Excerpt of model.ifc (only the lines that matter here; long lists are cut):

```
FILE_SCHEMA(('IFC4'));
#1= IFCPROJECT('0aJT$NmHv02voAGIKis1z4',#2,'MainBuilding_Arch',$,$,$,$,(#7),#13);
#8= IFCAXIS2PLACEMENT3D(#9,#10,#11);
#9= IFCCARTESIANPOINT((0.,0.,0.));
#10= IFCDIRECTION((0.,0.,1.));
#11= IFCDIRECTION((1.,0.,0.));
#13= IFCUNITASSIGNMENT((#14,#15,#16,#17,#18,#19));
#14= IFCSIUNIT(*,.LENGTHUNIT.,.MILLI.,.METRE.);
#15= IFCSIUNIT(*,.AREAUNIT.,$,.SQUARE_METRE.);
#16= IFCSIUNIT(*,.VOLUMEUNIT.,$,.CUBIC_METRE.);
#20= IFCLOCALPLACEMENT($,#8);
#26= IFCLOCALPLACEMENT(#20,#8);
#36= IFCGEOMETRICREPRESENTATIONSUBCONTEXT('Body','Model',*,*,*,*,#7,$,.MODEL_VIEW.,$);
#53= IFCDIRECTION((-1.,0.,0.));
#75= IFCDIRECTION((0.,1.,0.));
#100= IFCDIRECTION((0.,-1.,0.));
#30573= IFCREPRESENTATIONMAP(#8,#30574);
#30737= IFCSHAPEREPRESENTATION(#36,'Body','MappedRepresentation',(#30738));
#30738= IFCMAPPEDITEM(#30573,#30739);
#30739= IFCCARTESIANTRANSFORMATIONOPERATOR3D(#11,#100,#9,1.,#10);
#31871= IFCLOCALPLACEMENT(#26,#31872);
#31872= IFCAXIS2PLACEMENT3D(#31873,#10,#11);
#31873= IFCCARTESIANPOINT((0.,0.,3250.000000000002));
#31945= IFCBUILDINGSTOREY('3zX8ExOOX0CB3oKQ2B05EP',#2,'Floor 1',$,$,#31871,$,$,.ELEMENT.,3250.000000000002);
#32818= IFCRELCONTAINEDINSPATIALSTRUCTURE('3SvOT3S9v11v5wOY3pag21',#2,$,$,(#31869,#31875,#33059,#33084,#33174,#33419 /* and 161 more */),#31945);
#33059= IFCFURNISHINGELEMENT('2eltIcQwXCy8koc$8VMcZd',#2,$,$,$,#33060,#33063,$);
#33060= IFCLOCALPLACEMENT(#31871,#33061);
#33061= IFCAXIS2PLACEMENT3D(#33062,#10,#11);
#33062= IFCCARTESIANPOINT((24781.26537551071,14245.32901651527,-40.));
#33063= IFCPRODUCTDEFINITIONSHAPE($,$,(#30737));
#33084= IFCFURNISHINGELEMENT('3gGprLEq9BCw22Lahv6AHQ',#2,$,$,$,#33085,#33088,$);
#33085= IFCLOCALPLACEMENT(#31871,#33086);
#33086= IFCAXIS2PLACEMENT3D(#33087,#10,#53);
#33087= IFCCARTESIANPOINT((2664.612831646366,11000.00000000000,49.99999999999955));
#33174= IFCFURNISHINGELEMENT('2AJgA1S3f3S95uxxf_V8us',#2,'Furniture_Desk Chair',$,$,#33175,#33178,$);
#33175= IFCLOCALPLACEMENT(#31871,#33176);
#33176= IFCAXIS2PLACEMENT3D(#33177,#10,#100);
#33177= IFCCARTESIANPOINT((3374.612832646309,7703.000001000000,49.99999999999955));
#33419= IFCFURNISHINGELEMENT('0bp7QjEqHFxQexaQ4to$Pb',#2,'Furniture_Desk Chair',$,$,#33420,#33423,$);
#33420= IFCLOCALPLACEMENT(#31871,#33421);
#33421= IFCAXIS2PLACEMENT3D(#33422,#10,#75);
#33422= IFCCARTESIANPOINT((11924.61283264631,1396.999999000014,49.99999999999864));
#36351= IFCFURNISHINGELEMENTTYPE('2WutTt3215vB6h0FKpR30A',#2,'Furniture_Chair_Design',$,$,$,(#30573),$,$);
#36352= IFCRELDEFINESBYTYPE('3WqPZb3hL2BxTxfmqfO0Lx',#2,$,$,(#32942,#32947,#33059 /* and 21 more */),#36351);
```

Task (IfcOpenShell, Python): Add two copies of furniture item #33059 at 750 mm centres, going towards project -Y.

```python
import numpy as np
import ifcopenshell
import ifcopenshell.api.geometry
import ifcopenshell.api.root
import ifcopenshell.util.element
import ifcopenshell.util.placement

model = ifcopenshell.open("model.ifc")

source = model.by_id(33059)
base = ifcopenshell.util.placement.get_local_placement(source.ObjectPlacement)
step = np.array([0.0, -1.0, 0.0]) * 750.0

for i in range(1, 3):
    copy = ifcopenshell.api.root.copy_class(model, product=source)
    copy.Representation = ifcopenshell.util.element.copy_deep(
        model, source.Representation, exclude=["IfcGeometricRepresentationContext", "IfcRepresentationMap"]
    )
    matrix = base.copy()
    matrix[:3, 3] += i * step
    print("added at", matrix[:3, 3].round(3) + 0.0)
    ifcopenshell.api.geometry.edit_object_placement(model, product=copy, matrix=matrix, is_si=False)

model.write("model_edited.ifc")
```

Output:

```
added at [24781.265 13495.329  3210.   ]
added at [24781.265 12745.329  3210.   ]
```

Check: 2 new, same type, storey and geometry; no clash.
